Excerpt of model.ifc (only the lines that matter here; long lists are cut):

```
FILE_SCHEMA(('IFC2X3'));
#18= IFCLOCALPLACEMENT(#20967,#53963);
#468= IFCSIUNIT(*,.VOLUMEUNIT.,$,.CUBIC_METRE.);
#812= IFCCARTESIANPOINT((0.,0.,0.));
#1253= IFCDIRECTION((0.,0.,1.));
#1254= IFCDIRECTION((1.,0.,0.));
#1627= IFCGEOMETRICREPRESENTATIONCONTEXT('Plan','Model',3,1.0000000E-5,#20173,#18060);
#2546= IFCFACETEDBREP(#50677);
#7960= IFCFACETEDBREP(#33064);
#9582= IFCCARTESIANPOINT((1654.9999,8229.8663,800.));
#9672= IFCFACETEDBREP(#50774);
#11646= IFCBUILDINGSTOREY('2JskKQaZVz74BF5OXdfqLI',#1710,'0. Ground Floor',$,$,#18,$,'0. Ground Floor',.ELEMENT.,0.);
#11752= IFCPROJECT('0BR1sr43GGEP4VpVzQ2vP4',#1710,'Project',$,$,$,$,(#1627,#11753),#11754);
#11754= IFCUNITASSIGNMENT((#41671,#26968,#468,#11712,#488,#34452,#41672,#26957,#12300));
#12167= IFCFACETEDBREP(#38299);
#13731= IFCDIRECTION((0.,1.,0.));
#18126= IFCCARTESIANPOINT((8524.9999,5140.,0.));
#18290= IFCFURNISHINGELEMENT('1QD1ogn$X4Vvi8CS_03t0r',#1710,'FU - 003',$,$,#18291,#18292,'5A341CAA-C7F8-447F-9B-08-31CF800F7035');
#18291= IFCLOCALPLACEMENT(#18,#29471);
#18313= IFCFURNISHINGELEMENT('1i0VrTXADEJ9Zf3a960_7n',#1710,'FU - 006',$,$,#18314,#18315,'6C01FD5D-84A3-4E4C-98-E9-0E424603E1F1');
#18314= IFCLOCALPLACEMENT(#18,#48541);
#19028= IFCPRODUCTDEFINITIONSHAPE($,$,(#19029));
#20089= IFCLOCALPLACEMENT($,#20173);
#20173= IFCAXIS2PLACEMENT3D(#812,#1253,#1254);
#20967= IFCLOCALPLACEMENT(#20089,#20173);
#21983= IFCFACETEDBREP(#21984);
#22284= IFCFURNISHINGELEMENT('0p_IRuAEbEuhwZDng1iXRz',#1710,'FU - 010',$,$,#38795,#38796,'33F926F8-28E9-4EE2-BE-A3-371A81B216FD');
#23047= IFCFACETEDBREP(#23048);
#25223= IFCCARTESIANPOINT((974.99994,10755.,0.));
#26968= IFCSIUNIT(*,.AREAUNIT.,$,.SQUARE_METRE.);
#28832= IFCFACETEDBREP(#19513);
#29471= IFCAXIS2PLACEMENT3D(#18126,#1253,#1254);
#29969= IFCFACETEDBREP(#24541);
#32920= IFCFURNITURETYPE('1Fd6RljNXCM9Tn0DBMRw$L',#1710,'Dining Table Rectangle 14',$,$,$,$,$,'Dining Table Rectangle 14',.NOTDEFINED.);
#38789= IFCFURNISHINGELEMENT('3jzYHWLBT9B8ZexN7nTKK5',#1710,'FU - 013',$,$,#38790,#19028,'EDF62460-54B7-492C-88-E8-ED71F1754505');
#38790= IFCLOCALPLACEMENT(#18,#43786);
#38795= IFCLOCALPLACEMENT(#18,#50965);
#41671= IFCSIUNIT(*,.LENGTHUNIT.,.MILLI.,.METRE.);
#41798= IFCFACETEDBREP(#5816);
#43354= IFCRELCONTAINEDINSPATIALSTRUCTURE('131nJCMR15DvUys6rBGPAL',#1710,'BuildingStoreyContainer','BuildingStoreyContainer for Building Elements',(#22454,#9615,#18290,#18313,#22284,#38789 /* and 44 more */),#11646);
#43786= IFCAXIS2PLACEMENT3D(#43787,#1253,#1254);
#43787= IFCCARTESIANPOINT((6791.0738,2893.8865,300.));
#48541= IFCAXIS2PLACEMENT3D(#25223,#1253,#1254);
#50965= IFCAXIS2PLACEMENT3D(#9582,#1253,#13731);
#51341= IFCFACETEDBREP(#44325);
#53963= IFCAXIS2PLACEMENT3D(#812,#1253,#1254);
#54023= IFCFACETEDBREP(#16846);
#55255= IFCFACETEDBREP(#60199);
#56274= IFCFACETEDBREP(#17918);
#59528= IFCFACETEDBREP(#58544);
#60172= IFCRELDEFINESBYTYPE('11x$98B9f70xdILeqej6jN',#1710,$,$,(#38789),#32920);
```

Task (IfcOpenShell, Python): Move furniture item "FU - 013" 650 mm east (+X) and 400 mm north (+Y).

```python
import ifcopenshell
import ifcopenshell.api.geometry
import ifcopenshell.util.placement

model = ifcopenshell.open("model.ifc")

item = model.by_guid("3jzYHWLBT9B8ZexN7nTKK5")
matrix = ifcopenshell.util.placement.get_local_placement(item.ObjectPlacement)
matrix[0, 3] += 650.0
matrix[1, 3] += 400.0
ifcopenshell.api.geometry.edit_object_placement(model, product=item, matrix=matrix, is_si=False)

print(ifcopenshell.util.placement.get_local_placement(item.ObjectPlacement).round(3) + 0.0)

model.write("model_v2.ifc")
```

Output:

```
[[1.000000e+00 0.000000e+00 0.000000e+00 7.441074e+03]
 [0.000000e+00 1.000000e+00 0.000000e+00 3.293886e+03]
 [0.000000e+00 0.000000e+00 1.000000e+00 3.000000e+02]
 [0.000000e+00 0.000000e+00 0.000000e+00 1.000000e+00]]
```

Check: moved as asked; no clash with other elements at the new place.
